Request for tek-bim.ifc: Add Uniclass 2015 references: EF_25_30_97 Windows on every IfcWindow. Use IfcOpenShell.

First a look at what the model holds.

```python
import ifcopenshell

model = ifcopenshell.open("tek-bim.ifc")
print(model.schema)
print("classifications:", [c.Name for c in model.by_type("IfcClassification")])
for ifc_class in ("IfcDoor", "IfcRoof", "IfcStair", "IfcWall", "IfcWindow"):
    print(ifc_class, len(model.by_type(ifc_class)))
```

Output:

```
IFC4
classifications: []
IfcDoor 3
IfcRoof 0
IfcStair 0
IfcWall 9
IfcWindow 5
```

```python
import ifcopenshell
import ifcopenshell.api.classification

model = ifcopenshell.open("tek-bim.ifc")

system = ifcopenshell.api.classification.add_classification(model, classification="Uniclass 2015")

codes = {
    "IfcWindow": ("EF_25_30_97", "Windows"),
}
for ifc_class, (code, name) in codes.items():
    products = model.by_type(ifc_class)
    ifcopenshell.api.classification.add_reference(
        model, products=products, classification=system, identification=code, name=name
    )
    print(code, len(products))

model.write("tek-bim_v2.ifc")
```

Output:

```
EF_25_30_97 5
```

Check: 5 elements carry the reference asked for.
